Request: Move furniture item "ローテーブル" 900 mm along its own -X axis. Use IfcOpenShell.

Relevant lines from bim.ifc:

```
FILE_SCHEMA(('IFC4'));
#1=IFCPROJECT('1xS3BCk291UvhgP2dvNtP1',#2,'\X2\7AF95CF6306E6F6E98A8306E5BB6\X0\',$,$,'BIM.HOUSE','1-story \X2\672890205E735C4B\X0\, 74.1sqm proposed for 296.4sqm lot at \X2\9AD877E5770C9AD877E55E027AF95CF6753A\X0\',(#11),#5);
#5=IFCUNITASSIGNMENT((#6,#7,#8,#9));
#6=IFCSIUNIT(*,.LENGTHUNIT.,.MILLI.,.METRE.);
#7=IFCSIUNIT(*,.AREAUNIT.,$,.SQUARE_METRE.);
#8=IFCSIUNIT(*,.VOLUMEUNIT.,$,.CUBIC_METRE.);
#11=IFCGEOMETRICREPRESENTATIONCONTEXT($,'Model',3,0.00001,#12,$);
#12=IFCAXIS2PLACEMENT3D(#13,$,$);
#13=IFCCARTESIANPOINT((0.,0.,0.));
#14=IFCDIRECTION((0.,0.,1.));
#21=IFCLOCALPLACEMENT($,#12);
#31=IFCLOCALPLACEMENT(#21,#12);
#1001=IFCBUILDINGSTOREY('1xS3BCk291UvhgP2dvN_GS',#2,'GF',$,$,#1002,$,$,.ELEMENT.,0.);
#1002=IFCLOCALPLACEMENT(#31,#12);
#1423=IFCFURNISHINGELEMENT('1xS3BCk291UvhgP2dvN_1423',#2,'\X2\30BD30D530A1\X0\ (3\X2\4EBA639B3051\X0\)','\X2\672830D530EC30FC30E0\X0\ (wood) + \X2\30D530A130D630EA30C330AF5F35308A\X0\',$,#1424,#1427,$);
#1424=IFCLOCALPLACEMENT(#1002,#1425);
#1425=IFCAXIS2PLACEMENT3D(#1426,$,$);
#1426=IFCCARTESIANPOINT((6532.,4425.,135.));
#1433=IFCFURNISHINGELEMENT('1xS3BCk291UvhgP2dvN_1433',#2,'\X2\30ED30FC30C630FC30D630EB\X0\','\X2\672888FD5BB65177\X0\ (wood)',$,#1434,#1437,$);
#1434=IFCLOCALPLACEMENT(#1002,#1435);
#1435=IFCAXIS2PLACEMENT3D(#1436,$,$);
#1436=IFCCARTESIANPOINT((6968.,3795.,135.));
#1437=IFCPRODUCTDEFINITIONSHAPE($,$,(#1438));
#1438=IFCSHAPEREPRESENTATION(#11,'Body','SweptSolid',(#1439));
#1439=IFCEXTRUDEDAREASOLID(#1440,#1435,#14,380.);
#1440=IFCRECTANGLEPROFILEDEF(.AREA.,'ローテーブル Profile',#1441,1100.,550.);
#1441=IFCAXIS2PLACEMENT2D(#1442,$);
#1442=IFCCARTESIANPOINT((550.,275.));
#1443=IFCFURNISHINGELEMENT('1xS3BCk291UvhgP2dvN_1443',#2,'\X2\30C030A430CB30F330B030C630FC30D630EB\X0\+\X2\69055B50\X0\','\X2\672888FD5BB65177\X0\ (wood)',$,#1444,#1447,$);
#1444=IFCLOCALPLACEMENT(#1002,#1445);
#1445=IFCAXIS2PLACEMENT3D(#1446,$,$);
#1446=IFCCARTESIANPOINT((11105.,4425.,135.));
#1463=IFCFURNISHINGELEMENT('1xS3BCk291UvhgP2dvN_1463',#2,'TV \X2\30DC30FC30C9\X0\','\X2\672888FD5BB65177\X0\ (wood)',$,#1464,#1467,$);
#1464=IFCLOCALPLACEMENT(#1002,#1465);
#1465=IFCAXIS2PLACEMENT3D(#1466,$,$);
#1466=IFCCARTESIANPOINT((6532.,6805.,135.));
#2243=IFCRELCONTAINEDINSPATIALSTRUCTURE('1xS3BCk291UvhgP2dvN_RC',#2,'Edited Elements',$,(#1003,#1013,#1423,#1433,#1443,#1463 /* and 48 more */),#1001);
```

```python
import ifcopenshell
import ifcopenshell.api.geometry
import ifcopenshell.util.placement
import ifcopenshell.util.unit

model = ifcopenshell.open("bim.ifc")
unit_scale = ifcopenshell.util.unit.calculate_unit_scale(model)

item = model.by_id(1433)
matrix = ifcopenshell.util.placement.get_local_placement(item.ObjectPlacement)
matrix[:3, 3] -= matrix[:3, 0] * 0.9 / unit_scale
ifcopenshell.api.geometry.edit_object_placement(model, product=item, matrix=matrix, is_si=False)

print(ifcopenshell.util.placement.get_local_placement(item.ObjectPlacement).round(3) + 0.0)

model.write("bim_rev.ifc")
```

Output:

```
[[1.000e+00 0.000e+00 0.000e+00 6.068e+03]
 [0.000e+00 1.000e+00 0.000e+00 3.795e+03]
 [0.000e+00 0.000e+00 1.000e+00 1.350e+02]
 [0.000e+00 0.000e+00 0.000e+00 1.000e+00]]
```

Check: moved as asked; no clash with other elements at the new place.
